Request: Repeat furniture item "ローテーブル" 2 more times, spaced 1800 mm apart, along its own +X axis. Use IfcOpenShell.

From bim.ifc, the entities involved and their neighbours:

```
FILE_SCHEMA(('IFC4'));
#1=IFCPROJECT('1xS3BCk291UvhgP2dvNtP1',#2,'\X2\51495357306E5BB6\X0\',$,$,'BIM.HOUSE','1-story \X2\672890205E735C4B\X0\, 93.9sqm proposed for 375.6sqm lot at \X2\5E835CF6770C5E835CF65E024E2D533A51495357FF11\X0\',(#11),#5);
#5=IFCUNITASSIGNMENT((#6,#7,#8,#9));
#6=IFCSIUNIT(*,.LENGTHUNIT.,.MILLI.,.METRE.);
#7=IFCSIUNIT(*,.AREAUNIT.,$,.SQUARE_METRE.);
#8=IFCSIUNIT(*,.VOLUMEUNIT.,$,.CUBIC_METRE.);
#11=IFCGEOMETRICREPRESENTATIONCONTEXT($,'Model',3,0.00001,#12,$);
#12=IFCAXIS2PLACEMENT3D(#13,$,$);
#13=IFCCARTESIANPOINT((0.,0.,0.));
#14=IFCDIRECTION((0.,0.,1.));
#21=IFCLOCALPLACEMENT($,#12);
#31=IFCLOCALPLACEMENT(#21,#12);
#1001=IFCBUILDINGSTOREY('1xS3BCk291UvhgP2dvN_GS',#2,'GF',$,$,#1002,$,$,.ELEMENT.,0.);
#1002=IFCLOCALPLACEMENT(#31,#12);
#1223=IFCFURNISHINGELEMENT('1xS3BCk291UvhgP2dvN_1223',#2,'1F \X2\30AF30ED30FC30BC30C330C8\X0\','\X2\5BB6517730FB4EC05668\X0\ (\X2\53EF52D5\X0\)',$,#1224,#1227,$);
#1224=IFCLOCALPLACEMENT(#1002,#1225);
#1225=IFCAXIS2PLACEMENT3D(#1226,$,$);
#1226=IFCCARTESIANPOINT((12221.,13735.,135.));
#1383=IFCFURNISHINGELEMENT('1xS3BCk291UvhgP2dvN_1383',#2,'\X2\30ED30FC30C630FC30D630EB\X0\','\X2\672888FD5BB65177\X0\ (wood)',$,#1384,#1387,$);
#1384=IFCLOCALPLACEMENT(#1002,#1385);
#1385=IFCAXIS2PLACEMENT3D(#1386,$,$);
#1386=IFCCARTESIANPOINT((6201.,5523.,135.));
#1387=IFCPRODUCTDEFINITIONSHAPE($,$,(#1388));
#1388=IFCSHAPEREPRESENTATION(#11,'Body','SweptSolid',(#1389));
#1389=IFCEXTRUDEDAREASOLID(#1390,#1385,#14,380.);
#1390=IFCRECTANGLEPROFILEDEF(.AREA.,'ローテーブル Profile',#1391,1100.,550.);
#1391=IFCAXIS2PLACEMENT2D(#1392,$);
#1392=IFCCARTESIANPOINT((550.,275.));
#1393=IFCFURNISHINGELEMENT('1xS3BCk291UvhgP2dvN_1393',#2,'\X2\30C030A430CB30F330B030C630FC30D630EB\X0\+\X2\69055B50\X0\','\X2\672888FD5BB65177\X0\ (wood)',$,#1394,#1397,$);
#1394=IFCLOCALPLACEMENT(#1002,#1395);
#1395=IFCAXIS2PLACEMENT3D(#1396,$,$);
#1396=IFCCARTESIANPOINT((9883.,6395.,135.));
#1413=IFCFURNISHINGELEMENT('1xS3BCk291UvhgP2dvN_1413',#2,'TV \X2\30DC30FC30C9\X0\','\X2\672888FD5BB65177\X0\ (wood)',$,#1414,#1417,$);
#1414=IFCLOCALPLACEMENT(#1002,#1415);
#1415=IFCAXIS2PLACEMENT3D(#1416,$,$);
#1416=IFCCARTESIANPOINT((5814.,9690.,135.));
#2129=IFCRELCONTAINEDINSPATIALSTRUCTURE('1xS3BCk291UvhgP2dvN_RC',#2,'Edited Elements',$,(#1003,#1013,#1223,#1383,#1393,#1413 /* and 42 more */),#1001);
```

```python
import ifcopenshell
import ifcopenshell.api.geometry
import ifcopenshell.api.root
import ifcopenshell.util.element
import ifcopenshell.util.placement

model = ifcopenshell.open("bim.ifc")


def reuse_history(source, copy):
    """copy_class also copies each property set's owner history, people and application; keep the originals."""
    for rel in copy.IsDefinedBy:
        if rel.is_a("IfcRelDefinesByProperties") and (history := rel.RelatingPropertyDefinition.OwnerHistory):
            rel.RelatingPropertyDefinition.OwnerHistory = source.OwnerHistory
            ifcopenshell.util.element.remove_deep2(model, history)


source = model.by_guid("1xS3BCk291UvhgP2dvN_1383")
base = ifcopenshell.util.placement.get_local_placement(source.ObjectPlacement)
step = base[:3, 0] * 1800.0

for i in range(1, 3):
    copy = ifcopenshell.api.root.copy_class(model, product=source)
    copy.Representation = ifcopenshell.util.element.copy_deep(
        model, source.Representation, exclude=["IfcGeometricRepresentationContext", "IfcRepresentationMap"]
    )
    reuse_history(source, copy)
    matrix = base.copy()
    matrix[:3, 3] += i * step
    print("added at", matrix[:3, 3].round(3) + 0.0)
    ifcopenshell.api.geometry.edit_object_placement(model, product=copy, matrix=matrix, is_si=False)

model.write("bim-out.ifc")
```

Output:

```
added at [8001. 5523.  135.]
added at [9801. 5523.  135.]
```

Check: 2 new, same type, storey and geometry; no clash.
